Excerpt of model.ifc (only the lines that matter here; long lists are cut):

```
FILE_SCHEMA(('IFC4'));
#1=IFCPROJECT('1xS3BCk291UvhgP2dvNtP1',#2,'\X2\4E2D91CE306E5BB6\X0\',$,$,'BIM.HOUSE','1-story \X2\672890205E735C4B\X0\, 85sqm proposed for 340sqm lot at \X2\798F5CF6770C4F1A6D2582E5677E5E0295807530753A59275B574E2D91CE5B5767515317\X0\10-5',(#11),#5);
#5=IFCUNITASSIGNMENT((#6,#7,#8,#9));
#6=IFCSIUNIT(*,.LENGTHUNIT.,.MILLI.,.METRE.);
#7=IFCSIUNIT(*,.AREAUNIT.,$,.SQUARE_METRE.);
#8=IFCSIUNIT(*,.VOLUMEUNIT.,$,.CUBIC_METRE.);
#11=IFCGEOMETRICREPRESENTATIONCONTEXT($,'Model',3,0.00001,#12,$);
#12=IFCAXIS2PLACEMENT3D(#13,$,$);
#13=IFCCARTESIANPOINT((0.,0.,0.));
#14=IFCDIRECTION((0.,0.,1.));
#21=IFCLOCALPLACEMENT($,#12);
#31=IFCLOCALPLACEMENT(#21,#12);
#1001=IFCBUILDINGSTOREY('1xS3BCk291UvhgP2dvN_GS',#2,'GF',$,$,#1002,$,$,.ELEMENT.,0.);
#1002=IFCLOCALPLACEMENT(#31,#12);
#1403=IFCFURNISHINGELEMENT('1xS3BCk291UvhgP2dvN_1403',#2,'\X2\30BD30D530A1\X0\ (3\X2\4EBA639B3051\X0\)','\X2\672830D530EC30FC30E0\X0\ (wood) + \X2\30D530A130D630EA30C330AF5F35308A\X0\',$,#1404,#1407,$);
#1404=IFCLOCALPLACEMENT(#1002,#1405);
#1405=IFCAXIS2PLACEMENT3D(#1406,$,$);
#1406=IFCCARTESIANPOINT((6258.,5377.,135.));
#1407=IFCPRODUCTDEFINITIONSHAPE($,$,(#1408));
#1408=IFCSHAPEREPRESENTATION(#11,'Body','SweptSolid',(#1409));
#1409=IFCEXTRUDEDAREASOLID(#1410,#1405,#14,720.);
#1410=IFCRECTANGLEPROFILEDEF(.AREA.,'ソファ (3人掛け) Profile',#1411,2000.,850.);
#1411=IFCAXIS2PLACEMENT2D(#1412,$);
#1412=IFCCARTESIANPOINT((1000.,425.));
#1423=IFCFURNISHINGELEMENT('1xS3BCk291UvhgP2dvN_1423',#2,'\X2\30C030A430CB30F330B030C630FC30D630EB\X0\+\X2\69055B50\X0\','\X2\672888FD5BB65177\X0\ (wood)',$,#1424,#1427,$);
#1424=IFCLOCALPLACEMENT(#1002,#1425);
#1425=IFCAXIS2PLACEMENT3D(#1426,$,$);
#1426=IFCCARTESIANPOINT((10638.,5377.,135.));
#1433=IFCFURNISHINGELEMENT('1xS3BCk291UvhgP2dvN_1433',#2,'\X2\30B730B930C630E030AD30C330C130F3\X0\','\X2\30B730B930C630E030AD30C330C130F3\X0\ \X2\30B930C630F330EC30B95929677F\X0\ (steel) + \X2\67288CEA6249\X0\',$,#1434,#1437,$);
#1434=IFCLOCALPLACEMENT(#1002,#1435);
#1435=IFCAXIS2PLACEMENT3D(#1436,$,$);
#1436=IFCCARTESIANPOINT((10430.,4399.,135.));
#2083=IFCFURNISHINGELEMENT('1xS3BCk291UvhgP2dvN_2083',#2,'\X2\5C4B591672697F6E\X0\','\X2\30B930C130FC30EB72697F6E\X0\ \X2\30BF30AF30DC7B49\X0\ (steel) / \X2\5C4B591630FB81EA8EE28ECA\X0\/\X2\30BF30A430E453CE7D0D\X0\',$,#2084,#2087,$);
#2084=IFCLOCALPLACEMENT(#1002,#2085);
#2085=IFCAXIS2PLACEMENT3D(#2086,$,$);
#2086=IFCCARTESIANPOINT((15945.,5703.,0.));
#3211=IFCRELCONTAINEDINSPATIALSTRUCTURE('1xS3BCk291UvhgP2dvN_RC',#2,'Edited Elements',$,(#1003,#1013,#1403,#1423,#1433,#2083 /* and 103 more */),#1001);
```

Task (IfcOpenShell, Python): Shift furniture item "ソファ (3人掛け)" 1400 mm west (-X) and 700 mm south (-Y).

```python
import ifcopenshell
import ifcopenshell.api.geometry
import ifcopenshell.util.placement

model = ifcopenshell.open("model.ifc")

item = model.by_guid("1xS3BCk291UvhgP2dvN_1403")
matrix = ifcopenshell.util.placement.get_local_placement(item.ObjectPlacement)
matrix[0, 3] -= 1400.0
matrix[1, 3] -= 700.0
ifcopenshell.api.geometry.edit_object_placement(model, product=item, matrix=matrix, is_si=False)

print(ifcopenshell.util.placement.get_local_placement(item.ObjectPlacement).round(3) + 0.0)

model.write("model_v2.ifc")
```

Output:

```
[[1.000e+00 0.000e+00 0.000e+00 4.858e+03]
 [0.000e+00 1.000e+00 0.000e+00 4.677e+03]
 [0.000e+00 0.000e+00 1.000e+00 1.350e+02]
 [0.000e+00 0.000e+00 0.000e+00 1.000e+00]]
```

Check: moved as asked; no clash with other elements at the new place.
